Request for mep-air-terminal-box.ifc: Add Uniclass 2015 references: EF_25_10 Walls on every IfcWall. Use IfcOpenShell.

First a look at what the model holds.

```python
import ifcopenshell

model = ifcopenshell.open("mep-air-terminal-box.ifc")
print(model.schema)
print("classifications:", [c.Name for c in model.by_type("IfcClassification")])
for ifc_class in ("IfcDoor", "IfcRoof", "IfcStair", "IfcWall", "IfcWindow"):
    print(ifc_class, len(model.by_type(ifc_class)))
```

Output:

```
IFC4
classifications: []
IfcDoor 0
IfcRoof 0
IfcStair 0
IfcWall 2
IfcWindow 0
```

```python
import ifcopenshell
import ifcopenshell.api.classification

model = ifcopenshell.open("mep-air-terminal-box.ifc")

system = ifcopenshell.api.classification.add_classification(model, classification="Uniclass 2015")

codes = {
    "IfcWall": ("EF_25_10", "Walls"),
}
for ifc_class, (code, name) in codes.items():
    products = model.by_type(ifc_class)
    ifcopenshell.api.classification.add_reference(
        model, products=products, classification=system, identification=code, name=name
    )
    print(code, len(products))

model.write("mep-air-terminal-box_rev.ifc")
```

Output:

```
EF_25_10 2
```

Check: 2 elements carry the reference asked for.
